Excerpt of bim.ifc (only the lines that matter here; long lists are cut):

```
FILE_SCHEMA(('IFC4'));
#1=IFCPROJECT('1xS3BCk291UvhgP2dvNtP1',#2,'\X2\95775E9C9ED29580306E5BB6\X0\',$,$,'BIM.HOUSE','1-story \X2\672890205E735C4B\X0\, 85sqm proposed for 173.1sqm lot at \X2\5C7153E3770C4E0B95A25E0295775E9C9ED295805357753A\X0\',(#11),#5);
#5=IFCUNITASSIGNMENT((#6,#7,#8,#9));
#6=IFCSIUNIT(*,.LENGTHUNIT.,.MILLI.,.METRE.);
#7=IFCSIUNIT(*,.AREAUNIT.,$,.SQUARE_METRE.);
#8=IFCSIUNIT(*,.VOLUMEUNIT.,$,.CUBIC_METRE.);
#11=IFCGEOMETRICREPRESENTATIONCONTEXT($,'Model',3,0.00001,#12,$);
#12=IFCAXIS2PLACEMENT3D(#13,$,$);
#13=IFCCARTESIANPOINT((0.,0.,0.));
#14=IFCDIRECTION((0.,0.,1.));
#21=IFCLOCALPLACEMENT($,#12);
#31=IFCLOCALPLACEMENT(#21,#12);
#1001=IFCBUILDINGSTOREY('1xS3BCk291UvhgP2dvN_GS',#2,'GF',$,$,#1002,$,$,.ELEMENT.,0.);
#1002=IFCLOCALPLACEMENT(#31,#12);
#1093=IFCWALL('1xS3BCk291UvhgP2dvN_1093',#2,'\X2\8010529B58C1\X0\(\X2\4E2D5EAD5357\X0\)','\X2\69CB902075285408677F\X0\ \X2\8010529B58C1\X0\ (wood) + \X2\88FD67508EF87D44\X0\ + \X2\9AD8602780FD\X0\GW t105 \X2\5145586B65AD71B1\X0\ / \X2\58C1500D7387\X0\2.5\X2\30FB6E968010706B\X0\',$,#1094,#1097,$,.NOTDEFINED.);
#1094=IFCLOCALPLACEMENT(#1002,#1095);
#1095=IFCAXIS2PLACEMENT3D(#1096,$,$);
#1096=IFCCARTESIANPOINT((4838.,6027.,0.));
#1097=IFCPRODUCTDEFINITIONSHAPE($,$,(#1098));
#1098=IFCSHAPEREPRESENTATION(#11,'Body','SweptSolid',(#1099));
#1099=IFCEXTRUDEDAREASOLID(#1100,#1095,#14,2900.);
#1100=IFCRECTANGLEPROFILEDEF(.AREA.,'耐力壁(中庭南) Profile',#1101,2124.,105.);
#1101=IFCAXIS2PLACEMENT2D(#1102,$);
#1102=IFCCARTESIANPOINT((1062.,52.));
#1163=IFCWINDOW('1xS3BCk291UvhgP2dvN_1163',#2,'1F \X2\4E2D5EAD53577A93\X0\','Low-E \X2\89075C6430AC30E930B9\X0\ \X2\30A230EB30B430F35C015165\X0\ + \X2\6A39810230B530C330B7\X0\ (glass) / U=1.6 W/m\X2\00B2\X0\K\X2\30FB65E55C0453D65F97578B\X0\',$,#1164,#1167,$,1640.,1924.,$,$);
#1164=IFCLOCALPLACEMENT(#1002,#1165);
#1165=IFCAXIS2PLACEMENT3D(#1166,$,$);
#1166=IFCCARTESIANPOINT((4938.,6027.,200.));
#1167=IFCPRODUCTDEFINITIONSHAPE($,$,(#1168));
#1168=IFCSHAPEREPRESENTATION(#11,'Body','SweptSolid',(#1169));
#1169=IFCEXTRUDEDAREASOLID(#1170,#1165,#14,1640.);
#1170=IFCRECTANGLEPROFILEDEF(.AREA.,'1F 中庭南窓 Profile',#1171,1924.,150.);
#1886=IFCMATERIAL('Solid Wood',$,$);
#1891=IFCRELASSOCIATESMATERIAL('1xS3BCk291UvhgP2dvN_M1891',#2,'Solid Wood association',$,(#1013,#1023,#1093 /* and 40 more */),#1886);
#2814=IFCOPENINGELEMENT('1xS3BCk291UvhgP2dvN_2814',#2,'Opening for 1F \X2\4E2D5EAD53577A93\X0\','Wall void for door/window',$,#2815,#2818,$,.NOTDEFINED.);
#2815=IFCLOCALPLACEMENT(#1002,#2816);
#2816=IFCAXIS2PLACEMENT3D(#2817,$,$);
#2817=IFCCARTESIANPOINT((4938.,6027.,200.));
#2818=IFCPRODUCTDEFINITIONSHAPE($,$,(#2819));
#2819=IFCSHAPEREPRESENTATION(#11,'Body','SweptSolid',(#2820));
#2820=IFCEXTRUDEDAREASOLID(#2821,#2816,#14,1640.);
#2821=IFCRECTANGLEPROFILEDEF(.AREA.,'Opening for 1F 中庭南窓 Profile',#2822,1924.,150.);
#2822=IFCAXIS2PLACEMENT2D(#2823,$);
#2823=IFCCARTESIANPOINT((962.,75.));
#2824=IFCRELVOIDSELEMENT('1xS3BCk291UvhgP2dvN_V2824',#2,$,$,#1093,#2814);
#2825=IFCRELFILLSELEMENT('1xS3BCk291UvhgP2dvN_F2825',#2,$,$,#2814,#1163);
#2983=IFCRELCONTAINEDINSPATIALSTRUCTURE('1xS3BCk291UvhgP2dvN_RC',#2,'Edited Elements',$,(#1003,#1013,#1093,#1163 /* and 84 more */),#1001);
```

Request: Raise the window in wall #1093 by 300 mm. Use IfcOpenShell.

```python
import numpy as np
import ifcopenshell
import ifcopenshell.api.geometry
import ifcopenshell.util.placement
import ifcopenshell.util.unit

model = ifcopenshell.open("bim.ifc")
unit_scale = ifcopenshell.util.unit.calculate_unit_scale(model)

window = model.by_id(1163)
opening = window.FillsVoids[0].RelatingOpeningElement
dz = 0.3 / unit_scale

shift = np.array([0.0, 0.0, dz])
# The window is not placed relative to its opening, so move both.
for product in (opening, window):
    matrix = ifcopenshell.util.placement.get_local_placement(product.ObjectPlacement)
    matrix[:3, 3] += shift
    ifcopenshell.api.geometry.edit_object_placement(model, product=product, matrix=matrix, is_si=False)

print(f"moved by {dz * unit_scale:+.3f} m")

model.write("bim_edited.ifc")
```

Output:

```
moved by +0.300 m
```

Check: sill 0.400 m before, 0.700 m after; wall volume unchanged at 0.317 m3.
